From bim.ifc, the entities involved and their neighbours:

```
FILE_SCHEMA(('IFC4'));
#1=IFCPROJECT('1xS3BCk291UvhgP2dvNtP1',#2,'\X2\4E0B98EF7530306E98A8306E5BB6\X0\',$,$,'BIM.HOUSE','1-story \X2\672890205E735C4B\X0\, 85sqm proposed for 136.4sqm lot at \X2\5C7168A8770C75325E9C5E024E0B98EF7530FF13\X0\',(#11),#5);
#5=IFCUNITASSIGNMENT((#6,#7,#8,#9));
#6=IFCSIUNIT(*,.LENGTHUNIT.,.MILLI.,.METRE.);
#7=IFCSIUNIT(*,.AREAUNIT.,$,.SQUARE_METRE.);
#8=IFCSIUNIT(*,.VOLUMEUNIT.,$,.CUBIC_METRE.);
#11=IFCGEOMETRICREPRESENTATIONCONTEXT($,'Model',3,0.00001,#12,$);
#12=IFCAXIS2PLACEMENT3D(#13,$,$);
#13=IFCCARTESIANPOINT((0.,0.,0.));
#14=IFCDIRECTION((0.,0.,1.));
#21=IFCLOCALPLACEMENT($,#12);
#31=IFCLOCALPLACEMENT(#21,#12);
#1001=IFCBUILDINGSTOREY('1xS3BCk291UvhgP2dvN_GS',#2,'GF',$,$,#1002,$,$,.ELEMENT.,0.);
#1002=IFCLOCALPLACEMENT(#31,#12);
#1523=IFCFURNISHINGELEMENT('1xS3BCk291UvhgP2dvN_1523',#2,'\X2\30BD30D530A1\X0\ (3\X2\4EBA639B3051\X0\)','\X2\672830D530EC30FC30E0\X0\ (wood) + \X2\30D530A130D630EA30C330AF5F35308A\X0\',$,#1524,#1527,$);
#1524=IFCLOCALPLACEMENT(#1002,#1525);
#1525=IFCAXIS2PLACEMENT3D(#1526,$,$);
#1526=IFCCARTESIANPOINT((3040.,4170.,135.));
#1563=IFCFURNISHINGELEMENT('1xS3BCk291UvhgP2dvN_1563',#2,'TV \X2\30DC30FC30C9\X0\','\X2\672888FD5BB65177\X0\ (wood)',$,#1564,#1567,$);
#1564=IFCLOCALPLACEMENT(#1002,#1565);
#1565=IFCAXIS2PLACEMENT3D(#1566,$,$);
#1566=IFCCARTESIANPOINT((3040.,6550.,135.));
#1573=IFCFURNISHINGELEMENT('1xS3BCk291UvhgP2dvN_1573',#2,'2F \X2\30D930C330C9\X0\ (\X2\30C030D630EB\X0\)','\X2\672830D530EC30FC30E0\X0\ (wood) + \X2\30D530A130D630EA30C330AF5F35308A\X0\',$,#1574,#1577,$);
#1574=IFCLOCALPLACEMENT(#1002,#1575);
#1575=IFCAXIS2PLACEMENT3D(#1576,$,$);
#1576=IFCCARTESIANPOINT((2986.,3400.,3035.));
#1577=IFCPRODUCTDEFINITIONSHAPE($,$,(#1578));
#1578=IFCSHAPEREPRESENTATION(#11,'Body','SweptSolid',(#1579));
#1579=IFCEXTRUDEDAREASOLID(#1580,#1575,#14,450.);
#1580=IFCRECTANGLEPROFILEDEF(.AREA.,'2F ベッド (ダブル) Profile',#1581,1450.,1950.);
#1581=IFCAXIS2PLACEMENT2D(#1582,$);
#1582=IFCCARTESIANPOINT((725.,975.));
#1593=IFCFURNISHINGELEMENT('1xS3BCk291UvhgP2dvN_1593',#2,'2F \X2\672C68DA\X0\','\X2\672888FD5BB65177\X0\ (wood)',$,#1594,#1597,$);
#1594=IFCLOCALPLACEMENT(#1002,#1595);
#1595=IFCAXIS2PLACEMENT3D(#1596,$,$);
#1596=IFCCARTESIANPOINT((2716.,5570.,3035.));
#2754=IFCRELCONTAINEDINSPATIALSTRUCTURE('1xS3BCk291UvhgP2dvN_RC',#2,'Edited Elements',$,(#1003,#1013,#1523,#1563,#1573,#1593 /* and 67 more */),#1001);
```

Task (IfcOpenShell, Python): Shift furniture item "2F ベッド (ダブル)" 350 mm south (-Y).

```python
import ifcopenshell
import ifcopenshell.api.geometry
import ifcopenshell.util.placement
import ifcopenshell.util.unit

model = ifcopenshell.open("bim.ifc")
unit_scale = ifcopenshell.util.unit.calculate_unit_scale(model)

item = model.by_guid("1xS3BCk291UvhgP2dvN_1573")
matrix = ifcopenshell.util.placement.get_local_placement(item.ObjectPlacement)
matrix[1, 3] -= 0.35 / unit_scale
ifcopenshell.api.geometry.edit_object_placement(model, product=item, matrix=matrix, is_si=False)

print(ifcopenshell.util.placement.get_local_placement(item.ObjectPlacement).round(3) + 0.0)

model.write("bim-out.ifc")
```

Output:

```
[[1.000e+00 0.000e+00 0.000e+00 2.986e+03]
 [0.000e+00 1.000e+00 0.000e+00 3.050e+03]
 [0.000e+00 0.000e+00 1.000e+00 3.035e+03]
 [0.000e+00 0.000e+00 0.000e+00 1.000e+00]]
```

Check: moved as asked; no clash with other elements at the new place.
